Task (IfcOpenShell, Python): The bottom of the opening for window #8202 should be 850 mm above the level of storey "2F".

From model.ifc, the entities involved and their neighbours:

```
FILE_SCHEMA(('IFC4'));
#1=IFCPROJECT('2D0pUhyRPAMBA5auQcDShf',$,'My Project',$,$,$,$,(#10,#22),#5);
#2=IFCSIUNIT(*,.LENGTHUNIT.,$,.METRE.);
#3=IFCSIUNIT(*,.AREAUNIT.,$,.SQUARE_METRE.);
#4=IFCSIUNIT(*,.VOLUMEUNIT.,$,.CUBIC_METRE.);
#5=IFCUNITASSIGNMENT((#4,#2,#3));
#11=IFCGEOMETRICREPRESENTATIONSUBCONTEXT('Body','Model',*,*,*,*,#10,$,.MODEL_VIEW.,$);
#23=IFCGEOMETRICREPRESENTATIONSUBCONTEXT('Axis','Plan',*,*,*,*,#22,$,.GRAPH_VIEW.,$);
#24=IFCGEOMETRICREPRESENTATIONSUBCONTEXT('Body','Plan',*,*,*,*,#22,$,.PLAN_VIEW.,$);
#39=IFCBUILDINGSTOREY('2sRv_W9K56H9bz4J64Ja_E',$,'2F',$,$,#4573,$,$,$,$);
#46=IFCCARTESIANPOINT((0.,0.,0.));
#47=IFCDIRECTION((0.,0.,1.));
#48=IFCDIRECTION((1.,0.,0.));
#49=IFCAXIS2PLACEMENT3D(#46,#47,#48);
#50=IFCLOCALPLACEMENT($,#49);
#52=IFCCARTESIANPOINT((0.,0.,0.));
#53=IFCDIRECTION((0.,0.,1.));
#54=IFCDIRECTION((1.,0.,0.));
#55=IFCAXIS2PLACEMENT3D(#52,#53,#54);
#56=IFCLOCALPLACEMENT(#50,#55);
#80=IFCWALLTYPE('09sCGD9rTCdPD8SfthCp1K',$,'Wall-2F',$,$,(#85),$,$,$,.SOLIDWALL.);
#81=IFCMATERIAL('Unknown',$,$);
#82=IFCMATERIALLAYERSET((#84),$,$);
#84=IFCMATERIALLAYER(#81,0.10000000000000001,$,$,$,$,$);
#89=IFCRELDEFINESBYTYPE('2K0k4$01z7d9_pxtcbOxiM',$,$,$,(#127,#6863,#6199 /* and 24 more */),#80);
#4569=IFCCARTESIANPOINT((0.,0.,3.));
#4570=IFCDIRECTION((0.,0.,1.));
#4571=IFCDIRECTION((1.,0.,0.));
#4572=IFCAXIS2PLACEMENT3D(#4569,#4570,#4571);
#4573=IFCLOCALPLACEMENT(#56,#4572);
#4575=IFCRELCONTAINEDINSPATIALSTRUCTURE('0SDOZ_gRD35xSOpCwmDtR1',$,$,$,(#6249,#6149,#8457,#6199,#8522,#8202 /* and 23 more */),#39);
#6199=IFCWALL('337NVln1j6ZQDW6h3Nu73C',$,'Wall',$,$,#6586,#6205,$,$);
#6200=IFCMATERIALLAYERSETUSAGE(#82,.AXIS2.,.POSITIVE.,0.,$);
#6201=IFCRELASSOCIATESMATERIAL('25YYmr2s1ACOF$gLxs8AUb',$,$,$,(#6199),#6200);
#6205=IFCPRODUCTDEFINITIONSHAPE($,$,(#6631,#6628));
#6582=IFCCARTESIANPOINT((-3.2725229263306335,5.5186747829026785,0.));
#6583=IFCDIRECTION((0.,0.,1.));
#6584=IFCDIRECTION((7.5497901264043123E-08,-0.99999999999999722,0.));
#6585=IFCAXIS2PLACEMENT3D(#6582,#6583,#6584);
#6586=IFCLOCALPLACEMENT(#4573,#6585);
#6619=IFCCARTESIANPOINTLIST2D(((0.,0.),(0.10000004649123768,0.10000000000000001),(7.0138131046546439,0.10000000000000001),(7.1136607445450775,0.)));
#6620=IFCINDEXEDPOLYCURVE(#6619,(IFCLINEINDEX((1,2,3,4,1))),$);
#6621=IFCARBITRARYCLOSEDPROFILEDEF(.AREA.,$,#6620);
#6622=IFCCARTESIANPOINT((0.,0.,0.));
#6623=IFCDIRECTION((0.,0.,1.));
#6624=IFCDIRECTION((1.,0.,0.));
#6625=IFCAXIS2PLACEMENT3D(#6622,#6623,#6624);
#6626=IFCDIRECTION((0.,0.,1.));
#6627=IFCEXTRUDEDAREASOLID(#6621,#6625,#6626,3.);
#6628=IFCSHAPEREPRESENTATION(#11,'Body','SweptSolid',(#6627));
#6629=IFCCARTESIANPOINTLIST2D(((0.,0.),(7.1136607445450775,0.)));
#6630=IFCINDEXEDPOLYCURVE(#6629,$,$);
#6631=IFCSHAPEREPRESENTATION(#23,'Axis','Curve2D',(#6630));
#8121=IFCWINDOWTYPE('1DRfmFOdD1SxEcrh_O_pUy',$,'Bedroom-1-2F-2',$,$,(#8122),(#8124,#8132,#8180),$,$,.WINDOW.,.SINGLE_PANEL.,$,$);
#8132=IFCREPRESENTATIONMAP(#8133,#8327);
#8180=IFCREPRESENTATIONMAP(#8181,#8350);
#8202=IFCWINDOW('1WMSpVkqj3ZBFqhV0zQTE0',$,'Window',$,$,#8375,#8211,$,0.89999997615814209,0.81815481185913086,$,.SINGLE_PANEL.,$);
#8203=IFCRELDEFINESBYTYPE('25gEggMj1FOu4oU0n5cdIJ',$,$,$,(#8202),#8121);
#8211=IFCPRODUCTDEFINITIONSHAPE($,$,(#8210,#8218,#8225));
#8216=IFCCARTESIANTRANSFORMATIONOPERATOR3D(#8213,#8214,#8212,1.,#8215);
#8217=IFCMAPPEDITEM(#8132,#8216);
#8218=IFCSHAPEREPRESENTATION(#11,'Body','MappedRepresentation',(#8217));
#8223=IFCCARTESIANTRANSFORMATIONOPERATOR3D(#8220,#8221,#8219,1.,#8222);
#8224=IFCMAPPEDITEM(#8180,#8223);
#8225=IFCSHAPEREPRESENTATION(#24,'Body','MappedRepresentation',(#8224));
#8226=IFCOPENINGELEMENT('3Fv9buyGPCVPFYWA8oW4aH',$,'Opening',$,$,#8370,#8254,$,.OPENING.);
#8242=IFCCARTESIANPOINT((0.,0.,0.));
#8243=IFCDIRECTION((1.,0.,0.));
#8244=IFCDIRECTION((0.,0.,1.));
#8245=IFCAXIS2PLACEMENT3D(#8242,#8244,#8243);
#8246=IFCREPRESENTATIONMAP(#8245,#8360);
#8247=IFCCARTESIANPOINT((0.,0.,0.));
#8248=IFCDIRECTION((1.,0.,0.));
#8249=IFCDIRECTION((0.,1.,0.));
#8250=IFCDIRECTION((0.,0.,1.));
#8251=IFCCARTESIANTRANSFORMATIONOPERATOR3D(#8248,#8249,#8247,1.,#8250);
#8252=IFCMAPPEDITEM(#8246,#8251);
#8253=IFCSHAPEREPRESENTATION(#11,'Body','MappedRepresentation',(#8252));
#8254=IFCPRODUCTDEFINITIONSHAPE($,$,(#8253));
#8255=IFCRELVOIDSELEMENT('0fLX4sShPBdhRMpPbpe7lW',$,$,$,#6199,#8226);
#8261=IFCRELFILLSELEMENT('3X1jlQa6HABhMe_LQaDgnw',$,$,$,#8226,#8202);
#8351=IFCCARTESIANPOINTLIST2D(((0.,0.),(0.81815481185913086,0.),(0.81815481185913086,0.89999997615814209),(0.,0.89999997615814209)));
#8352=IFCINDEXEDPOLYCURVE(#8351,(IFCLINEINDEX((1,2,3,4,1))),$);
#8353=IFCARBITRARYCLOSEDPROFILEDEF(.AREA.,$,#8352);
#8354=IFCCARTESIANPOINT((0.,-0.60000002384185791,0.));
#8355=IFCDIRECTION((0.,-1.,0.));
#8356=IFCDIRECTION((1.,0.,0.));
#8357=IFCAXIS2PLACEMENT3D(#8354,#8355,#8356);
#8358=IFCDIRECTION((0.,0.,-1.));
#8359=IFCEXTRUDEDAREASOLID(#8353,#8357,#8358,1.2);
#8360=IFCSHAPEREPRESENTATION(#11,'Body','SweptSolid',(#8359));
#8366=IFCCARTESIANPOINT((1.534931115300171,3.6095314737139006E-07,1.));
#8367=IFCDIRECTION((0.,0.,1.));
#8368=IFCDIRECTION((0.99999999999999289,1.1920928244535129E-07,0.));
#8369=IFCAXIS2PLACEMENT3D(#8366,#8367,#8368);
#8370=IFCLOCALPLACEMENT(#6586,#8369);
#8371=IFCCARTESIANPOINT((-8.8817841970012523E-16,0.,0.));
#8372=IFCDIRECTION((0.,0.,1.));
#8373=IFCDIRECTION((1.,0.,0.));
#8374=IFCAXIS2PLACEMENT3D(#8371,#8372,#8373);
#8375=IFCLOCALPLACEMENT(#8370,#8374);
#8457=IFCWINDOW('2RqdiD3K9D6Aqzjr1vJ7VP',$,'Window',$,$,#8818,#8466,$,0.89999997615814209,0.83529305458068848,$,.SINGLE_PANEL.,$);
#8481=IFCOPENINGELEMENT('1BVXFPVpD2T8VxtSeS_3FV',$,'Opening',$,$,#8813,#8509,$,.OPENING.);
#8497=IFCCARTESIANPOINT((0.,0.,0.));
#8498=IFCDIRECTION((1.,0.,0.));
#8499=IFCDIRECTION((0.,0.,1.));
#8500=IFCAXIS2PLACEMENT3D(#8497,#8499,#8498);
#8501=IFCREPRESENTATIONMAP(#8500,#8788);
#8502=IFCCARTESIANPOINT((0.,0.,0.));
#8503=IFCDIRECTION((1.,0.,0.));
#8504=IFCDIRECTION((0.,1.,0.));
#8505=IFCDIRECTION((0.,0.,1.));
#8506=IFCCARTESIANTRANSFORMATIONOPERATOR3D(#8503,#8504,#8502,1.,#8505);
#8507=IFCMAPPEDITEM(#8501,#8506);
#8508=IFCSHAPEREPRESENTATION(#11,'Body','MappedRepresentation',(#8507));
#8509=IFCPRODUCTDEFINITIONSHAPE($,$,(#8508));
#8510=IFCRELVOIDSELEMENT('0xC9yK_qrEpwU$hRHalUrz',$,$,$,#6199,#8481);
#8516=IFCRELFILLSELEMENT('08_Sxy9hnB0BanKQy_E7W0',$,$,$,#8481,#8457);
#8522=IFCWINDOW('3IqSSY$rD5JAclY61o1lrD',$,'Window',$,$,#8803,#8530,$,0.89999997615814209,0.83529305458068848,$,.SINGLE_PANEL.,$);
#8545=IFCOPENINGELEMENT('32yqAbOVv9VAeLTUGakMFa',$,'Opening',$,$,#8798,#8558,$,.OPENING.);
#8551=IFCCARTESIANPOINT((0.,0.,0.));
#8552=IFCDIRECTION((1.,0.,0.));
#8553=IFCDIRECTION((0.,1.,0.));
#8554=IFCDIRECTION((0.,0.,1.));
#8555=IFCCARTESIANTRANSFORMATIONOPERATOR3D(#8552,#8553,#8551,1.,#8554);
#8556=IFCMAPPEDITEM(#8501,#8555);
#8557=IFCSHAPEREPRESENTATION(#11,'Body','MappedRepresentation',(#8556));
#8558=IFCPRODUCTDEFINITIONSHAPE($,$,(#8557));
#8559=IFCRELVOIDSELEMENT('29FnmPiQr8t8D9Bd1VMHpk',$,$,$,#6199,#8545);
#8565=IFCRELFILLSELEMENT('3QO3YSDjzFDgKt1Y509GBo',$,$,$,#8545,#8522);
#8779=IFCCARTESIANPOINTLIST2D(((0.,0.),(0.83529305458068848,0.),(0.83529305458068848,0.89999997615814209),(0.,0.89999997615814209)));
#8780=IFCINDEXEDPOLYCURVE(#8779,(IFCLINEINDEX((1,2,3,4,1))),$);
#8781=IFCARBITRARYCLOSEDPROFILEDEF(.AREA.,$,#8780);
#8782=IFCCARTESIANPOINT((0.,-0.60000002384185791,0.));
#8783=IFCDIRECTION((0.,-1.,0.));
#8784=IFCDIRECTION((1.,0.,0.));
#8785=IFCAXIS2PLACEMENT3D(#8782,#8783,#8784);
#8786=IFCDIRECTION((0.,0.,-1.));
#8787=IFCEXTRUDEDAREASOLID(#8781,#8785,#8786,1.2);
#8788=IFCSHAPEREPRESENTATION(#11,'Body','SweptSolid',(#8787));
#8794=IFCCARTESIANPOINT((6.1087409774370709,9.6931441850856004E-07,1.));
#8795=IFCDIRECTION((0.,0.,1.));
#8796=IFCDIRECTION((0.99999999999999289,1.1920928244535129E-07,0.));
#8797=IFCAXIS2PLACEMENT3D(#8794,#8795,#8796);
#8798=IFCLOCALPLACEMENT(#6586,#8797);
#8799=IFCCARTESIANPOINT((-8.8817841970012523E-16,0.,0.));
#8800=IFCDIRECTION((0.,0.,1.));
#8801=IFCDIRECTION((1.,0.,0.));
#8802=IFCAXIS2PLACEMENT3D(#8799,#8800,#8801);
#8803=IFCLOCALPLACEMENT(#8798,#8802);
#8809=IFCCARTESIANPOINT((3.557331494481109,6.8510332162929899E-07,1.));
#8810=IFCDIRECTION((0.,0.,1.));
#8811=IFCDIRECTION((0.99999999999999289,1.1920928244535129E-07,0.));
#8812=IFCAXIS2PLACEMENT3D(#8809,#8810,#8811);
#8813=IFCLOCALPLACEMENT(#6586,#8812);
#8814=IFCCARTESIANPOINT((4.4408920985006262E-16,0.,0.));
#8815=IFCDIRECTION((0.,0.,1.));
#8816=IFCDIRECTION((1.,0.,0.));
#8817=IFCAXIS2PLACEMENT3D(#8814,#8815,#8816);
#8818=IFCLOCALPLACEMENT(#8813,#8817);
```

```python
import numpy as np
import ifcopenshell
import ifcopenshell.api.geometry
import ifcopenshell.geom
import ifcopenshell.util.element
import ifcopenshell.util.placement
import ifcopenshell.util.shape
import ifcopenshell.util.unit

model = ifcopenshell.open("model.ifc")
unit_scale = ifcopenshell.util.unit.calculate_unit_scale(model)

window = model.by_guid("1WMSpVkqj3ZBFqhV0zQTE0")
opening = window.FillsVoids[0].RelatingOpeningElement
storey = ifcopenshell.util.element.get_container(window, ifc_class="IfcBuildingStorey")
level = ifcopenshell.util.placement.get_local_placement(storey.ObjectPlacement)[2, 3]

# The opening's origin need not be at the sill, so measure its lowest point.
shape = ifcopenshell.geom.create_shape(ifcopenshell.geom.settings(), opening)
bottom = ifcopenshell.util.shape.get_shape_bottom_elevation(shape, shape.geometry) / unit_scale
dz = level + 0.85 / unit_scale - bottom

shift = np.array([0.0, 0.0, dz])
# The window is placed relative to its opening, so it follows when the opening moves.
matrix = ifcopenshell.util.placement.get_local_placement(opening.ObjectPlacement)
matrix[:3, 3] += shift
ifcopenshell.api.geometry.edit_object_placement(
    model, product=opening, matrix=matrix, is_si=False, should_transform_children=True
)

print(f"moved by {dz * unit_scale:+.3f} m")

model.write("model_updated.ifc")
```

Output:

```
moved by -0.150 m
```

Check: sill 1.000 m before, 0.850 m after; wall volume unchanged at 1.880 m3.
